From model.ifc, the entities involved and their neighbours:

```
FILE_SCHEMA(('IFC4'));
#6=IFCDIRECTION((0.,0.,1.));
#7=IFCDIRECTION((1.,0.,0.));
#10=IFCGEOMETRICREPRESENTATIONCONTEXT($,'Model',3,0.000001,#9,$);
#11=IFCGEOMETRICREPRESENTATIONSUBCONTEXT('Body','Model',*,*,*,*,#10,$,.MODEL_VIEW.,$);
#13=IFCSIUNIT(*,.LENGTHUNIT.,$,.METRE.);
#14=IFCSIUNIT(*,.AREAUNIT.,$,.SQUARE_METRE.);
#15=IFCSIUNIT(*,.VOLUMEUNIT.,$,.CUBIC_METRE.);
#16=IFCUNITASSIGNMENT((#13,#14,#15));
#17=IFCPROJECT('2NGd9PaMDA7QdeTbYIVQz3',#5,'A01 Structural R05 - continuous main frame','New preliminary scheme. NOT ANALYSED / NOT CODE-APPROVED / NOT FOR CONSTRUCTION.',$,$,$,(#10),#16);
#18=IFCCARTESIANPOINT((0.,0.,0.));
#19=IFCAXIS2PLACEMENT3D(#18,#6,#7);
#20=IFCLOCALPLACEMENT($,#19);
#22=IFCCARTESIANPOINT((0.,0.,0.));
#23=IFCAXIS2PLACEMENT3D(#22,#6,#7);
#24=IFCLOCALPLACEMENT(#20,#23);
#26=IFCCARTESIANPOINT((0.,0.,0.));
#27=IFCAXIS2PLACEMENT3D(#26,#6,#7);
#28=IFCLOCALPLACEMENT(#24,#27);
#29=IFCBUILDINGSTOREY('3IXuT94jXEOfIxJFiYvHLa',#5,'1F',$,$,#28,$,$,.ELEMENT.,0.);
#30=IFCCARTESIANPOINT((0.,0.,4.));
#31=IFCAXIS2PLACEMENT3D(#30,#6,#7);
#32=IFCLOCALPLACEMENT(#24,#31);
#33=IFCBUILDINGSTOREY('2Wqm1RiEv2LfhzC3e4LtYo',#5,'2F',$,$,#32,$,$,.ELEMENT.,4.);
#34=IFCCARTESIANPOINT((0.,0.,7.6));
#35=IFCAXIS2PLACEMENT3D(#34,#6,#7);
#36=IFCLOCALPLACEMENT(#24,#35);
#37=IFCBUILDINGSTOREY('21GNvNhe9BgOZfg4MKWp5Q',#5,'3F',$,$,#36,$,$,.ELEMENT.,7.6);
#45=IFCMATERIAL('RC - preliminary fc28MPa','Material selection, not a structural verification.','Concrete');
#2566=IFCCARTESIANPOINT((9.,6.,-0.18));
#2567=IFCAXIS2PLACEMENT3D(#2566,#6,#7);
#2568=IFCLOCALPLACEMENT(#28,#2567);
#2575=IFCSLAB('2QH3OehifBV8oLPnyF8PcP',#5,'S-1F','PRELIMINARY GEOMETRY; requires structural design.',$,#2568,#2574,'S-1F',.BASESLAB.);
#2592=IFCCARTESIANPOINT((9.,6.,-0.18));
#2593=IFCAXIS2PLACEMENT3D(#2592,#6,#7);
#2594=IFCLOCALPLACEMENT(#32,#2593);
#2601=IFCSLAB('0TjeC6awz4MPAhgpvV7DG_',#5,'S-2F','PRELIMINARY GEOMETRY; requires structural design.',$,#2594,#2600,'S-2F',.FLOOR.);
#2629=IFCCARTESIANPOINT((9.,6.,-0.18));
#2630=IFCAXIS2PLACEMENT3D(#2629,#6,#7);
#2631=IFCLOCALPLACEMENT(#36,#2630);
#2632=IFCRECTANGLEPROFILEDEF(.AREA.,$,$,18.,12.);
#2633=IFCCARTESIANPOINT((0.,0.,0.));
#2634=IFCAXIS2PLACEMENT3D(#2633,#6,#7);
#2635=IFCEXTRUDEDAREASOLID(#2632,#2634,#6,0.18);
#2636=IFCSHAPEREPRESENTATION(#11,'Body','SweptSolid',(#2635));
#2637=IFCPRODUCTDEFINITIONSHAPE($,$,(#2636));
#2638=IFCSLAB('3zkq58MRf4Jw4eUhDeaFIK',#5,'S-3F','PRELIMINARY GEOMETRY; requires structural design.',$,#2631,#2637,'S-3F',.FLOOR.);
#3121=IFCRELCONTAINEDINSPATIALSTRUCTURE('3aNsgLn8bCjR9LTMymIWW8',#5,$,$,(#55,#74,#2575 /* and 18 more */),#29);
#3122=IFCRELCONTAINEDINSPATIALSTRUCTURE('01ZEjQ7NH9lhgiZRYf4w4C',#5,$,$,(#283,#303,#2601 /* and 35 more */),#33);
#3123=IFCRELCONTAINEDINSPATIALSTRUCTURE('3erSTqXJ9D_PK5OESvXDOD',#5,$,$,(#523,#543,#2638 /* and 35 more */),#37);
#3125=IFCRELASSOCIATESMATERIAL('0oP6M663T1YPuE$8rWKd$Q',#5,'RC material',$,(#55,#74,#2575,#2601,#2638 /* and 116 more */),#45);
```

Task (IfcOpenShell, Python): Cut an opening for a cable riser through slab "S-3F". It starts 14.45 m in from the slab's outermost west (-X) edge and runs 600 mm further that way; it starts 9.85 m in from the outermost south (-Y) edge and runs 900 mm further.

```python
import numpy as np
import ifcopenshell
import ifcopenshell.api.feature
import ifcopenshell.api.geometry
import ifcopenshell.api.root
import ifcopenshell.geom
import ifcopenshell.util.placement
import ifcopenshell.util.representation
import ifcopenshell.util.shape
import ifcopenshell.util.unit

model = ifcopenshell.open("model.ifc")
unit_scale = ifcopenshell.util.unit.calculate_unit_scale(model)
settings = ifcopenshell.geom.settings()


def volume(element):
    """Net volume in cubic metres, openings subtracted."""
    shape = ifcopenshell.geom.create_shape(settings, element)
    return ifcopenshell.util.shape.get_volume(shape.geometry)


slab = model.by_guid("3zkq58MRf4Jw4eUhDeaFIK")
before = volume(slab)

# Extent in the slab's own axes, in metres. The edges named are its -X and -Y sides.
slab_shape = ifcopenshell.geom.create_shape(settings, slab)
vertices = ifcopenshell.util.shape.get_vertices(slab_shape.geometry)
x_min, y_min, bottom = vertices.min(axis=0)
top = vertices[:, 2].max()

opening = ifcopenshell.api.root.create_entity(model, ifc_class="IfcOpeningElement", name="Cable riser opening", predefined_type="OPENING")
context = ifcopenshell.util.representation.get_context(model, "Model", "Body", "MODEL_VIEW")
width, depth = 0.6, 0.9
outline = [(0.0, 0.0), (width, 0.0), (width, depth), (0.0, depth), (0.0, 0.0)]
# Overshoot both faces by 50 mm so the cut is clean.
shape = ifcopenshell.api.geometry.add_slab_representation(
    model, context=context, depth=top - bottom + 0.1, polyline=outline
)
ifcopenshell.api.geometry.assign_representation(model, product=opening, representation=shape)

matrix = ifcopenshell.util.placement.get_local_placement(slab.ObjectPlacement)
matrix[:, 3] = matrix @ np.append(np.array([x_min + 14.45, y_min + 9.85, bottom - 0.05]) / unit_scale, 1.0)
ifcopenshell.api.geometry.edit_object_placement(model, product=opening, matrix=matrix, is_si=False)
ifcopenshell.api.feature.add_feature(model, feature=opening, element=slab)

after = volume(slab)

print(f"slab volume {before:.3f} -> {after:.3f} m3")

model.write("model_updated.ifc")
```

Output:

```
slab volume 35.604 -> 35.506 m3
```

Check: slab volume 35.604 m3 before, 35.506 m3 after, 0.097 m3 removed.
